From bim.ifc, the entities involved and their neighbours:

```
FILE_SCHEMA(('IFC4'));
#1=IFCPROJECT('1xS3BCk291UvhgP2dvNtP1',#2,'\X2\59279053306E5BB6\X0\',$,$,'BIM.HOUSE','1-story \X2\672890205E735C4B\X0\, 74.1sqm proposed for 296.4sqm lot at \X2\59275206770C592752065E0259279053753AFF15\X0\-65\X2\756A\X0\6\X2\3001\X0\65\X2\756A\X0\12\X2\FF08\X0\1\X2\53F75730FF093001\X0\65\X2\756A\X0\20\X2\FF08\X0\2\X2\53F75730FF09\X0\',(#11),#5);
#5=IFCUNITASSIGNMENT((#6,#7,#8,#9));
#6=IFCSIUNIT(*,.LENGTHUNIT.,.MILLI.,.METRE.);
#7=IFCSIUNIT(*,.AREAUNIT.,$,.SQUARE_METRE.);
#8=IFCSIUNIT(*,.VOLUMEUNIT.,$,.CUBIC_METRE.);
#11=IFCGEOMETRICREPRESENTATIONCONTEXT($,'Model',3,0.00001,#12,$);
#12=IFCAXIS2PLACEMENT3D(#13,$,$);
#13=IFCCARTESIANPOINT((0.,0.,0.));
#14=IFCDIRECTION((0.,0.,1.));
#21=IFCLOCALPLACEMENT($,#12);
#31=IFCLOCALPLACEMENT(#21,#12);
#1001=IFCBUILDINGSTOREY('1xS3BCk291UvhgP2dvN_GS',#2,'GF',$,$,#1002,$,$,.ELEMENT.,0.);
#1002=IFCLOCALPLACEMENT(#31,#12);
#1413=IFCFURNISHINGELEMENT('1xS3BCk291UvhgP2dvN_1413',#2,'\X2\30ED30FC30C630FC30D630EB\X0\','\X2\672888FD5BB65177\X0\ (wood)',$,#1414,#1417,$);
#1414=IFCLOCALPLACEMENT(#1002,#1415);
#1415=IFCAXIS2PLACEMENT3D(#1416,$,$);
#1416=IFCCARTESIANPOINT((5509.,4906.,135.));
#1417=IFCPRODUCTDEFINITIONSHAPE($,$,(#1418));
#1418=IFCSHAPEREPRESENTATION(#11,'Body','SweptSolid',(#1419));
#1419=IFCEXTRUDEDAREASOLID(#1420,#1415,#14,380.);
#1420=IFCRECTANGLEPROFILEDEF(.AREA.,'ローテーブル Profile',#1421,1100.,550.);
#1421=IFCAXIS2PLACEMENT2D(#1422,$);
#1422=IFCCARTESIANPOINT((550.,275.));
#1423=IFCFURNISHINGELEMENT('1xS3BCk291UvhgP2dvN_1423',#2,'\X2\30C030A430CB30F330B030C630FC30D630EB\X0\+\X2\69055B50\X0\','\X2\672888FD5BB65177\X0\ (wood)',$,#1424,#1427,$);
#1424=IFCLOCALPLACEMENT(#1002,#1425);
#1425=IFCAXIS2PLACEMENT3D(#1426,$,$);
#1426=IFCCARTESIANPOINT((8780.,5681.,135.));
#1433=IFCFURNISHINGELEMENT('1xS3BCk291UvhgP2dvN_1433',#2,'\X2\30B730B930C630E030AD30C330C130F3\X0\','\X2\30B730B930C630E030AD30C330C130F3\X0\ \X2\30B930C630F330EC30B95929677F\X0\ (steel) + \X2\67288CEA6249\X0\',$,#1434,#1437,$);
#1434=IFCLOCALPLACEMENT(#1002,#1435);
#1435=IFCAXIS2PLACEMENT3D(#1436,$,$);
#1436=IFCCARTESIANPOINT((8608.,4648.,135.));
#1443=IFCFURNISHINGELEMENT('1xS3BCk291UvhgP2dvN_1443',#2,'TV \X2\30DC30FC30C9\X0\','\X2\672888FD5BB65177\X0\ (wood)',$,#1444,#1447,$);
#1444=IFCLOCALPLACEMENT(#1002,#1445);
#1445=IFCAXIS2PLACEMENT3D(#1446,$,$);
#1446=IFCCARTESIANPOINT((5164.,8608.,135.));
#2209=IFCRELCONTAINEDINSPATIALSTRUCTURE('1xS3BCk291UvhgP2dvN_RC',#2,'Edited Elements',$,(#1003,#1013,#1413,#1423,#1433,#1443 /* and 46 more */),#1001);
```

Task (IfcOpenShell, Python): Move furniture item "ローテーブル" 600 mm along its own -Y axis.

```python
import ifcopenshell
import ifcopenshell.api.geometry
import ifcopenshell.util.placement
import ifcopenshell.util.unit

model = ifcopenshell.open("bim.ifc")
unit_scale = ifcopenshell.util.unit.calculate_unit_scale(model)

item = model.by_guid("1xS3BCk291UvhgP2dvN_1413")
matrix = ifcopenshell.util.placement.get_local_placement(item.ObjectPlacement)
matrix[:3, 3] -= matrix[:3, 1] * 0.6 / unit_scale
ifcopenshell.api.geometry.edit_object_placement(model, product=item, matrix=matrix, is_si=False)

print(ifcopenshell.util.placement.get_local_placement(item.ObjectPlacement).round(3) + 0.0)

model.write("bim_v2.ifc")
```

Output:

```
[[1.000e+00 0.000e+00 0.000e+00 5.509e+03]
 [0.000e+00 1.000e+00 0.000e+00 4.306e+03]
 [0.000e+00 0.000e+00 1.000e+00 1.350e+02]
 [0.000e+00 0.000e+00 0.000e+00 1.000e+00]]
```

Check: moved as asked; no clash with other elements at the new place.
